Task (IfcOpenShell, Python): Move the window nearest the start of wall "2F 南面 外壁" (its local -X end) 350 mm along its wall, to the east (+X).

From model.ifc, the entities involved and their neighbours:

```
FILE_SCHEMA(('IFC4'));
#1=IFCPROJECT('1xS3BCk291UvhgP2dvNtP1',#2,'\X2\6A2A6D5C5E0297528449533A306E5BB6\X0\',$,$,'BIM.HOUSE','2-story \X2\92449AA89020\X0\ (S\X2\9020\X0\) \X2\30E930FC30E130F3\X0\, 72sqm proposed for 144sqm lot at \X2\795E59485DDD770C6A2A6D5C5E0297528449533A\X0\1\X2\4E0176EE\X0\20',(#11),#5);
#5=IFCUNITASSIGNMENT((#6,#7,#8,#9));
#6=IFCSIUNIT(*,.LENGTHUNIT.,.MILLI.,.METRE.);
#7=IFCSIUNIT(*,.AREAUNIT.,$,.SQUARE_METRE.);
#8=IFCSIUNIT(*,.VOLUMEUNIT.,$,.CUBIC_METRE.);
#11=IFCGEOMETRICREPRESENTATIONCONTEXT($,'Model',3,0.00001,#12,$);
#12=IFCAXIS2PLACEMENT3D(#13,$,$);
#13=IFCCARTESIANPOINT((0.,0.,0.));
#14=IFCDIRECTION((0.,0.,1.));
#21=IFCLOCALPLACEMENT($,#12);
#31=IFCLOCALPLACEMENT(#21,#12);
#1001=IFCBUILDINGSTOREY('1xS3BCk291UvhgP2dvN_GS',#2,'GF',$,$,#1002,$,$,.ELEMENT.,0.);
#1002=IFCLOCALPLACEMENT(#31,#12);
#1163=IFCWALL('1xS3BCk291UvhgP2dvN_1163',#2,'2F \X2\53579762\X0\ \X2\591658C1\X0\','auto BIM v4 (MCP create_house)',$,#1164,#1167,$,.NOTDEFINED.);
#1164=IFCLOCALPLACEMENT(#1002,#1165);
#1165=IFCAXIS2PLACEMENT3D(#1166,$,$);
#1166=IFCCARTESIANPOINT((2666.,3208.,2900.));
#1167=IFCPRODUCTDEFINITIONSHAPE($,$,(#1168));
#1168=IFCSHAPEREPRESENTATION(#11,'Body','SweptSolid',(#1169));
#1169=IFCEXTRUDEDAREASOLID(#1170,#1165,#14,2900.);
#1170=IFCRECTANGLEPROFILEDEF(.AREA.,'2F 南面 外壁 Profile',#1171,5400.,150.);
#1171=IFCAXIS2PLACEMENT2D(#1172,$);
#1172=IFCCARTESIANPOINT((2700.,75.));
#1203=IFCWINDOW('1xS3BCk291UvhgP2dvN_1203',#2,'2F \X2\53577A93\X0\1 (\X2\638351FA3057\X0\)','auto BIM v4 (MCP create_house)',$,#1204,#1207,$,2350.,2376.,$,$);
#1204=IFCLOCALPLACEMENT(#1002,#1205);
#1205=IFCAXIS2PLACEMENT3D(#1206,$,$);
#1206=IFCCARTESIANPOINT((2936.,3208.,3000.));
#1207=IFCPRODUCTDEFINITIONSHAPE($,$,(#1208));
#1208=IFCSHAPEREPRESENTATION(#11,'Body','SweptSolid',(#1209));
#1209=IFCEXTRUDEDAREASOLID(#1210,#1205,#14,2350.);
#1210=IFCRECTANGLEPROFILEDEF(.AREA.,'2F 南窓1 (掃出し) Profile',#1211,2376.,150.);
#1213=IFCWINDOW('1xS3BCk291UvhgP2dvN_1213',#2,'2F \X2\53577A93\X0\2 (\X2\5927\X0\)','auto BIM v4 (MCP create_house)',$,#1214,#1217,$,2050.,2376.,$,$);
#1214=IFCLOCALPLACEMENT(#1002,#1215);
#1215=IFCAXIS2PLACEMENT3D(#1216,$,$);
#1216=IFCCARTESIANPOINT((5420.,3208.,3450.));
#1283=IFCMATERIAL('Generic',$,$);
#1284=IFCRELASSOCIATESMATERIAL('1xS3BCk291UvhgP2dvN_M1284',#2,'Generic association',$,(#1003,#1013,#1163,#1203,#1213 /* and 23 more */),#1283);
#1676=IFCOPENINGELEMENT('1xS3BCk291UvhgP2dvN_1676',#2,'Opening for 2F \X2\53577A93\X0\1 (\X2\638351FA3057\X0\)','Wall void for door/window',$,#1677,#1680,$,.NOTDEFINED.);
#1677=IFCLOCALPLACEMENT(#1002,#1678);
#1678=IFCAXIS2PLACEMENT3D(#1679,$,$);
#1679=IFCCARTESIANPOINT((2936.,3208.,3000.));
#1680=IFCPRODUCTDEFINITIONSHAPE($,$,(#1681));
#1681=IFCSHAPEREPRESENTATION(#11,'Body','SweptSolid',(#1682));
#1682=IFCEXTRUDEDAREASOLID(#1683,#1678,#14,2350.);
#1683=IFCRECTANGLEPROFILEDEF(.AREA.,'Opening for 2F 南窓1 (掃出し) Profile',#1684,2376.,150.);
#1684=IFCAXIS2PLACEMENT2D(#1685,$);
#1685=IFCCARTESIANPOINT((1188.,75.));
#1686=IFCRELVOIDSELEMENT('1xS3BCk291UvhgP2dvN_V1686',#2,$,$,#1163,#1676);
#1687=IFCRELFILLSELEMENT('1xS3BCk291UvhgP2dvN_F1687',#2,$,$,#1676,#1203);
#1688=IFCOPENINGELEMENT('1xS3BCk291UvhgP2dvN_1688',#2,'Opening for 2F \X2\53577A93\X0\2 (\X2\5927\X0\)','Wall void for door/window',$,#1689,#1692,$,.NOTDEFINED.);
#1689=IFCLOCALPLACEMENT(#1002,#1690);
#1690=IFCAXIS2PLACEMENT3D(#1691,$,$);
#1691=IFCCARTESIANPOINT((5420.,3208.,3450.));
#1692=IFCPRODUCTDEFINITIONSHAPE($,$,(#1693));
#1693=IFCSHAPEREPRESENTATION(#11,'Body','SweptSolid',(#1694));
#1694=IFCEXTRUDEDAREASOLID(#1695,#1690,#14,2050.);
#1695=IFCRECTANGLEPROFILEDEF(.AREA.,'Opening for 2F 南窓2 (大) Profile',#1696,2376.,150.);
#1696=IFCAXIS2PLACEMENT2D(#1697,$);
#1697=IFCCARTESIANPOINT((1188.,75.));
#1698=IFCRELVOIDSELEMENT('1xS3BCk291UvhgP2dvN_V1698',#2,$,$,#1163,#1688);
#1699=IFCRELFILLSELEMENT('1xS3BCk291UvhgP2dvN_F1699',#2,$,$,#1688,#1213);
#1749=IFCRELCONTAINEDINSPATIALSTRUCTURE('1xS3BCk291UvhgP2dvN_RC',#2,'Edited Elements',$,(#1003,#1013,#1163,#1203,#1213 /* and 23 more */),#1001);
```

```python
import ifcopenshell
import ifcopenshell.api.geometry
import ifcopenshell.util.placement

model = ifcopenshell.open("model.ifc")

window = model.by_id(1203)
opening = window.FillsVoids[0].RelatingOpeningElement
wall = opening.VoidsElements[0].RelatingBuildingElement

wall_matrix = ifcopenshell.util.placement.get_local_placement(wall.ObjectPlacement)
shift = wall_matrix[:3, 0] * 350.0
before = ifcopenshell.util.placement.get_local_placement(window.ObjectPlacement)[:3, 3].copy()

# The window is not placed relative to its opening, so move both.
for product in (opening, window):
    matrix = ifcopenshell.util.placement.get_local_placement(product.ObjectPlacement)
    matrix[:3, 3] += shift
    ifcopenshell.api.geometry.edit_object_placement(model, product=product, matrix=matrix, is_si=False)

after = ifcopenshell.util.placement.get_local_placement(window.ObjectPlacement)[:3, 3]
print("window moved by", (after - before).round(3) + 0.0)

model.write("model-out.ifc")
```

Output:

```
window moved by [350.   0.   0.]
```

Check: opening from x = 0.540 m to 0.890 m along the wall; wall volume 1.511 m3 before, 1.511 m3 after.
